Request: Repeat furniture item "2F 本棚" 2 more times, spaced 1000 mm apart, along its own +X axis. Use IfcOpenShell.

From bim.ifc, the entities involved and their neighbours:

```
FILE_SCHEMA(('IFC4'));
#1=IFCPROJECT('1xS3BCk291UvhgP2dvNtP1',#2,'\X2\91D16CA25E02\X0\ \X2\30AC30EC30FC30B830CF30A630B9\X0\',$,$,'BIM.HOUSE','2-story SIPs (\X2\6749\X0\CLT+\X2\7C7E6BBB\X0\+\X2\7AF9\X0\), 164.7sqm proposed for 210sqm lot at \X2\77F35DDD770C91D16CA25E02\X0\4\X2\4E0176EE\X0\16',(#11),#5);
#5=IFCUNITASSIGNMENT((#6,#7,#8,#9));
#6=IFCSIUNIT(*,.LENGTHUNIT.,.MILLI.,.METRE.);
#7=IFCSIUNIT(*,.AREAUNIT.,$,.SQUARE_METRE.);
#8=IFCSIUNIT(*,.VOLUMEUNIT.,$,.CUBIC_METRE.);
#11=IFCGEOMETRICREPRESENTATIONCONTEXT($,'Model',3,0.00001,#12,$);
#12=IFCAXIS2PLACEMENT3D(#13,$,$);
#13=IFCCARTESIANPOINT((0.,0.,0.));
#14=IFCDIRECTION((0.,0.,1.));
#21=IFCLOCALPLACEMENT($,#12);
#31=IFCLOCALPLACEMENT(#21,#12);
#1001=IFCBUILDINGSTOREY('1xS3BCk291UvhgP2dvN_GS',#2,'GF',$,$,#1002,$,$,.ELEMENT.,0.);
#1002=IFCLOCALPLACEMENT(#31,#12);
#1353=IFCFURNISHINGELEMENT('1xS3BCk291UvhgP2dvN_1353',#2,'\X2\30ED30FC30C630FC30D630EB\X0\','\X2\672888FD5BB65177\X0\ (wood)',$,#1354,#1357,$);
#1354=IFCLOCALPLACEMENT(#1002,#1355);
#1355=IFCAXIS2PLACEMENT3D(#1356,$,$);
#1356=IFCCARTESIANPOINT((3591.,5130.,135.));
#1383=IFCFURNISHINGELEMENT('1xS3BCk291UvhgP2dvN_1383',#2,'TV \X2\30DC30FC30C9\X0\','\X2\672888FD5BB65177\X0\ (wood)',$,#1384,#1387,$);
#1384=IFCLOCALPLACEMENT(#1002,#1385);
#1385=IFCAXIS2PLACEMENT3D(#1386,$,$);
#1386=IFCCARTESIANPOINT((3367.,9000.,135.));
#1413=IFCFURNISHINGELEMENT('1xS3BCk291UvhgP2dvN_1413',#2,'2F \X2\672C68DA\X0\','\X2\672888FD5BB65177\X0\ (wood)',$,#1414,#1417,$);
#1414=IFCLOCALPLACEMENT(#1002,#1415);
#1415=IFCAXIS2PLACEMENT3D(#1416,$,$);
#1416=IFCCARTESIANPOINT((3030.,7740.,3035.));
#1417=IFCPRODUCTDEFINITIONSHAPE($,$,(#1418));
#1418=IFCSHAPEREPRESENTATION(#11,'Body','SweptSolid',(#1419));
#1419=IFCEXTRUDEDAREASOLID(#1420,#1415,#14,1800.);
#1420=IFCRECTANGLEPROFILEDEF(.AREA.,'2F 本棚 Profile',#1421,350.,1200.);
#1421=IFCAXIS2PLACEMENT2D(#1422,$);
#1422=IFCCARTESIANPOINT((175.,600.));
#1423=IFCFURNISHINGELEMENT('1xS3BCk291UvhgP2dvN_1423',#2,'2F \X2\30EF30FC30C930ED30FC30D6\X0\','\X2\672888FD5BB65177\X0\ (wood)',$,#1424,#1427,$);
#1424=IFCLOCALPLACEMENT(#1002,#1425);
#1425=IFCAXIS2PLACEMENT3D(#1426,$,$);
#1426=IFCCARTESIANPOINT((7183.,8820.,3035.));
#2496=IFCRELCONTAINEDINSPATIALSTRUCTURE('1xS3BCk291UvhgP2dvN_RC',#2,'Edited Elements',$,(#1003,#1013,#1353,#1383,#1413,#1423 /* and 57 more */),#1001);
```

```python
import ifcopenshell
import ifcopenshell.api.geometry
import ifcopenshell.api.root
import ifcopenshell.util.element
import ifcopenshell.util.placement
import ifcopenshell.util.unit

model = ifcopenshell.open("bim.ifc")
unit_scale = ifcopenshell.util.unit.calculate_unit_scale(model)


def reuse_history(source, copy):
    """copy_class also copies each property set's owner history, people and application; keep the originals."""
    for rel in copy.IsDefinedBy:
        if rel.is_a("IfcRelDefinesByProperties") and (history := rel.RelatingPropertyDefinition.OwnerHistory):
            rel.RelatingPropertyDefinition.OwnerHistory = source.OwnerHistory
            ifcopenshell.util.element.remove_deep2(model, history)


source = model.by_guid("1xS3BCk291UvhgP2dvN_1413")
base = ifcopenshell.util.placement.get_local_placement(source.ObjectPlacement)
step = base[:3, 0] * 1 / unit_scale

for i in range(1, 3):
    copy = ifcopenshell.api.root.copy_class(model, product=source)
    copy.Representation = ifcopenshell.util.element.copy_deep(
        model, source.Representation, exclude=["IfcGeometricRepresentationContext", "IfcRepresentationMap"]
    )
    reuse_history(source, copy)
    matrix = base.copy()
    matrix[:3, 3] += i * step
    print("added at", matrix[:3, 3].round(3) + 0.0)
    ifcopenshell.api.geometry.edit_object_placement(model, product=copy, matrix=matrix, is_si=False)

model.write("bim_rev.ifc")
```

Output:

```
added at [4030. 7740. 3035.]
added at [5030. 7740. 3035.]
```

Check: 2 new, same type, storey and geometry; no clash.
